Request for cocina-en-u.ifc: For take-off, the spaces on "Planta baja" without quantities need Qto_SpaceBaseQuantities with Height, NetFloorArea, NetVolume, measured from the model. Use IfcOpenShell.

First a look at what the model holds.

```python
import ifcopenshell
import ifcopenshell.util.element
import ifcopenshell.util.unit

model = ifcopenshell.open("cocina-en-u.ifc")
print(model.schema)
for unit_type in ("LENGTHUNIT", "AREAUNIT", "VOLUMEUNIT"):
    print(unit_type, ifcopenshell.util.unit.calculate_unit_scale(model, unit_type))
storey = next(s for s in model.by_type("IfcBuildingStorey") if s.Name == "Planta baja")
spaces = [e for e in ifcopenshell.util.element.get_decomposition(storey) if e.is_a("IfcSpace")]
for e in sorted(spaces, key=lambda e: e.id()):
    print(e.id(), e.is_a(), e.Name, list(ifcopenshell.util.element.get_psets(e, qtos_only=True)), sep=" | ")
```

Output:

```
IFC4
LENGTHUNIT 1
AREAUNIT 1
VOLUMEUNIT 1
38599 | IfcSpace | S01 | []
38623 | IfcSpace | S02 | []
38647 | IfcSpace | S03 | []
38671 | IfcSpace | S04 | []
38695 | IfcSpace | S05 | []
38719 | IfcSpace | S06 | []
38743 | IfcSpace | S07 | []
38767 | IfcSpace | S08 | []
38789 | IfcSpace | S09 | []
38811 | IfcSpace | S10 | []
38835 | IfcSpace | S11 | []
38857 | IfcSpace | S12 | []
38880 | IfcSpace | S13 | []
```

```python
import ifcopenshell
import ifcopenshell.api.pset
import ifcopenshell.geom
import ifcopenshell.util.element
import ifcopenshell.util.shape
import ifcopenshell.util.unit

model = ifcopenshell.open("cocina-en-u.ifc")
unit_scale = ifcopenshell.util.unit.calculate_unit_scale(model)
area_scale = ifcopenshell.util.unit.calculate_unit_scale(model, "AREAUNIT")
volume_scale = ifcopenshell.util.unit.calculate_unit_scale(model, "VOLUMEUNIT")
settings = ifcopenshell.geom.settings()

storey = next(s for s in model.by_type("IfcBuildingStorey") if s.Name == "Planta baja")
spaces = [e for e in ifcopenshell.util.element.get_decomposition(storey) if e.is_a("IfcSpace")]

for e in sorted(spaces, key=lambda e: e.id()):
    if ifcopenshell.util.element.get_psets(e, qtos_only=True, should_inherit=False):
        continue
    # Geometry comes back in metres, in the element's own axes.
    shape = ifcopenshell.geom.create_shape(settings, e)
    values = {
        "Height": ifcopenshell.util.shape.get_z(shape.geometry) / unit_scale,
        "NetFloorArea": ifcopenshell.util.shape.get_footprint_area(shape.geometry) / area_scale,
        "NetVolume": ifcopenshell.util.shape.get_volume(shape.geometry) / volume_scale,
    }
    qto = ifcopenshell.api.pset.add_qto(model, product=e, name="Qto_SpaceBaseQuantities")
    ifcopenshell.api.pset.edit_qto(model, qto=qto, properties=values)
    print(e.id(), {k: round(v, 3) for k, v in values.items()})

model.write("cocina-en-u_v2.ifc")
```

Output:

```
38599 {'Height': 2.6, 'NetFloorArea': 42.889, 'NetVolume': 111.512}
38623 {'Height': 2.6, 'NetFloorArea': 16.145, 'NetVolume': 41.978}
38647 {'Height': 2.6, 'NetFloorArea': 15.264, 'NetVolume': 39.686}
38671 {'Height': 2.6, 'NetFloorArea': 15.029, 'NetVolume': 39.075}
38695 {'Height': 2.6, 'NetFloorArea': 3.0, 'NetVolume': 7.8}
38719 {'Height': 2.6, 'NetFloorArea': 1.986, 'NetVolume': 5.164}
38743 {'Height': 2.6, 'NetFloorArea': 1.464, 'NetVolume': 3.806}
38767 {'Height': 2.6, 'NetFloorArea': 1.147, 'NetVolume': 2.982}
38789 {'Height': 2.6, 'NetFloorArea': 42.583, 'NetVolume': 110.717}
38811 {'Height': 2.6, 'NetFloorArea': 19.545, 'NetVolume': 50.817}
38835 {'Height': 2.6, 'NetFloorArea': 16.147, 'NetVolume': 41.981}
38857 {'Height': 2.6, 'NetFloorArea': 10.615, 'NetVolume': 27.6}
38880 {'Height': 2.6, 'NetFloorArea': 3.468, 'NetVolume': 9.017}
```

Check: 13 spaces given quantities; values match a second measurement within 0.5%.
